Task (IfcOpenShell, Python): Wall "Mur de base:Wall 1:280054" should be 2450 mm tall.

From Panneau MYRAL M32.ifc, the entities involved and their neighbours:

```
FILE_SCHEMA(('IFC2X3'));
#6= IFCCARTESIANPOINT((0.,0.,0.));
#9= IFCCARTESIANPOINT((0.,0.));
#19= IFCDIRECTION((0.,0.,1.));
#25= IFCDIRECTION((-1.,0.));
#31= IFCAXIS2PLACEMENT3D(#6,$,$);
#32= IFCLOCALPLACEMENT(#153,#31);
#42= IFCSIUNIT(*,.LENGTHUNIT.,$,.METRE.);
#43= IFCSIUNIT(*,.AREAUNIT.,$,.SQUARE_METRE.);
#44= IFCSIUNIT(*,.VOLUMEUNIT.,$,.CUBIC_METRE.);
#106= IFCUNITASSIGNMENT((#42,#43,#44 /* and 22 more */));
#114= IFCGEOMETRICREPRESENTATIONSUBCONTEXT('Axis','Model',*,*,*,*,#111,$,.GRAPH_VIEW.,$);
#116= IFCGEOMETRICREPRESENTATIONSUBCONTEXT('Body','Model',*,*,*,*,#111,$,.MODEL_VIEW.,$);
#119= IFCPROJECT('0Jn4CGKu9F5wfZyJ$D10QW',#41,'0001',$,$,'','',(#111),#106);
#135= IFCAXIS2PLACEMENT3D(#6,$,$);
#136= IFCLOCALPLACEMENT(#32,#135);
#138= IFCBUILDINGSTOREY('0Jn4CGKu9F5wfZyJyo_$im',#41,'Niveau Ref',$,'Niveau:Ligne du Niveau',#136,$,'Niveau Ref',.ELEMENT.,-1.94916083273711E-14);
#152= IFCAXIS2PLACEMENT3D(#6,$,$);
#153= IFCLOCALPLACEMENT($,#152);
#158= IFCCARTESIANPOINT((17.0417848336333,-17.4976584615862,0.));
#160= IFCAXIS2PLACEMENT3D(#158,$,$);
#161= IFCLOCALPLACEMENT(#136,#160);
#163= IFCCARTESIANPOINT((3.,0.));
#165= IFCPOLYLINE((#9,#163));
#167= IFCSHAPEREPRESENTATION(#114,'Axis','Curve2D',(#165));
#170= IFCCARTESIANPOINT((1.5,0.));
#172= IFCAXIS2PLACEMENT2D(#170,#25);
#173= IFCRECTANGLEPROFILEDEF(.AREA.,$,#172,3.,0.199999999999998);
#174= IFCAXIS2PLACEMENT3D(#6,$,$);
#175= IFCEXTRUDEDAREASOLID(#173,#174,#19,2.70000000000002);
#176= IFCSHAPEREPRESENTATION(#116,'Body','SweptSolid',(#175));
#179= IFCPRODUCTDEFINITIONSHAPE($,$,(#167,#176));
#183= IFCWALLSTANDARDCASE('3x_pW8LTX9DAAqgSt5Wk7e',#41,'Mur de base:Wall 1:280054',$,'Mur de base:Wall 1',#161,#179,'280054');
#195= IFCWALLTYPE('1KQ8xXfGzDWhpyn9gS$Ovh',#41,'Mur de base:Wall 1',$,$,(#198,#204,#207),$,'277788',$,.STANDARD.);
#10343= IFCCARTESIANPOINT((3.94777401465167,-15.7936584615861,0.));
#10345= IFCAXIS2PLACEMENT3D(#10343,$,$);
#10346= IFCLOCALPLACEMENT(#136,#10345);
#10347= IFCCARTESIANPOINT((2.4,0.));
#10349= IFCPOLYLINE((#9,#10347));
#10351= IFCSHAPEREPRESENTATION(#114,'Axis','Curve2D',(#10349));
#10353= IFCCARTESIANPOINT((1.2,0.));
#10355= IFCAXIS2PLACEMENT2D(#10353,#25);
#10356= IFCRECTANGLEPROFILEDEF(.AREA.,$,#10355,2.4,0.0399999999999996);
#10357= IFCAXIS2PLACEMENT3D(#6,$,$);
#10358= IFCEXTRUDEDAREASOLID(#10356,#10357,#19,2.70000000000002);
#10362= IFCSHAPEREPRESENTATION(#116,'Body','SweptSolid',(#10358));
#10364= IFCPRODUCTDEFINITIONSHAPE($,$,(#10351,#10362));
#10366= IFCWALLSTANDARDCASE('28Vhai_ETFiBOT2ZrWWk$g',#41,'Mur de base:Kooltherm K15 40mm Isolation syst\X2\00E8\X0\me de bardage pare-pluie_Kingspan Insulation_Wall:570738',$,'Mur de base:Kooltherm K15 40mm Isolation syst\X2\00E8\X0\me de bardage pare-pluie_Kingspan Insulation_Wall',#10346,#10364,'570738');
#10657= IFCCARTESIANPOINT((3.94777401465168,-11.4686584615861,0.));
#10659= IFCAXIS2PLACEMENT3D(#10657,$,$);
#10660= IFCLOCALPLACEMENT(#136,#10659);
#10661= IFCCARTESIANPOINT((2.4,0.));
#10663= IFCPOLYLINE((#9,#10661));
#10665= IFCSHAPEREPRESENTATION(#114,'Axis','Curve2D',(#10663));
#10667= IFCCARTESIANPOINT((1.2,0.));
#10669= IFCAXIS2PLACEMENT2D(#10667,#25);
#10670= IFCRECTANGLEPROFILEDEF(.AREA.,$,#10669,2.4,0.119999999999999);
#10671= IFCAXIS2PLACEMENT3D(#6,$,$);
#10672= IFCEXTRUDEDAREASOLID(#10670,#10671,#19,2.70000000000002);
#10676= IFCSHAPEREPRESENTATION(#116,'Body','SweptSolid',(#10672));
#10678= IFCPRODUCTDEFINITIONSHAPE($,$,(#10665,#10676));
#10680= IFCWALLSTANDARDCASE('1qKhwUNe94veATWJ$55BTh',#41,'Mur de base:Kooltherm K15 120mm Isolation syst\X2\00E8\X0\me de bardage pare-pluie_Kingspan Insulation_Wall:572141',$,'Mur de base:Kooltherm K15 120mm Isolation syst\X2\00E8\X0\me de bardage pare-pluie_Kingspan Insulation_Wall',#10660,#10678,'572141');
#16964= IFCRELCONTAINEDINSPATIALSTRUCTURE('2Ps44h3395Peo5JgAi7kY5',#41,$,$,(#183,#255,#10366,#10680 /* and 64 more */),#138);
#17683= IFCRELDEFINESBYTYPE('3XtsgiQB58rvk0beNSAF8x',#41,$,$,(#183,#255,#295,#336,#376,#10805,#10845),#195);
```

```python
import ifcopenshell
import ifcopenshell.geom
import ifcopenshell.util.representation
import ifcopenshell.util.shape
import ifcopenshell.util.unit

model = ifcopenshell.open("Panneau MYRAL M32.ifc")
unit_scale = ifcopenshell.util.unit.calculate_unit_scale(model)
settings = ifcopenshell.geom.settings()


def volume(element):
    """Net volume in cubic metres, openings subtracted."""
    shape = ifcopenshell.geom.create_shape(settings, element)
    return ifcopenshell.util.shape.get_volume(shape.geometry)


wall = model.by_guid("3x_pW8LTX9DAAqgSt5Wk7e")
before = volume(wall)

body = ifcopenshell.util.representation.get_representation(wall, "Model", "Body")
solid = body.Items[0]
old_height = solid.Depth
solid.Depth = 2.45 / unit_scale
after = volume(wall)

print(f"height {old_height:g} -> {solid.Depth:g}, volume {before:.3f} -> {after:.3f} m3")

model.write("Panneau MYRAL M32_updated.ifc")
```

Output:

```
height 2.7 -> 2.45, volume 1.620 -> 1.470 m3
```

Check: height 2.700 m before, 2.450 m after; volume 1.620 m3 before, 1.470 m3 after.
